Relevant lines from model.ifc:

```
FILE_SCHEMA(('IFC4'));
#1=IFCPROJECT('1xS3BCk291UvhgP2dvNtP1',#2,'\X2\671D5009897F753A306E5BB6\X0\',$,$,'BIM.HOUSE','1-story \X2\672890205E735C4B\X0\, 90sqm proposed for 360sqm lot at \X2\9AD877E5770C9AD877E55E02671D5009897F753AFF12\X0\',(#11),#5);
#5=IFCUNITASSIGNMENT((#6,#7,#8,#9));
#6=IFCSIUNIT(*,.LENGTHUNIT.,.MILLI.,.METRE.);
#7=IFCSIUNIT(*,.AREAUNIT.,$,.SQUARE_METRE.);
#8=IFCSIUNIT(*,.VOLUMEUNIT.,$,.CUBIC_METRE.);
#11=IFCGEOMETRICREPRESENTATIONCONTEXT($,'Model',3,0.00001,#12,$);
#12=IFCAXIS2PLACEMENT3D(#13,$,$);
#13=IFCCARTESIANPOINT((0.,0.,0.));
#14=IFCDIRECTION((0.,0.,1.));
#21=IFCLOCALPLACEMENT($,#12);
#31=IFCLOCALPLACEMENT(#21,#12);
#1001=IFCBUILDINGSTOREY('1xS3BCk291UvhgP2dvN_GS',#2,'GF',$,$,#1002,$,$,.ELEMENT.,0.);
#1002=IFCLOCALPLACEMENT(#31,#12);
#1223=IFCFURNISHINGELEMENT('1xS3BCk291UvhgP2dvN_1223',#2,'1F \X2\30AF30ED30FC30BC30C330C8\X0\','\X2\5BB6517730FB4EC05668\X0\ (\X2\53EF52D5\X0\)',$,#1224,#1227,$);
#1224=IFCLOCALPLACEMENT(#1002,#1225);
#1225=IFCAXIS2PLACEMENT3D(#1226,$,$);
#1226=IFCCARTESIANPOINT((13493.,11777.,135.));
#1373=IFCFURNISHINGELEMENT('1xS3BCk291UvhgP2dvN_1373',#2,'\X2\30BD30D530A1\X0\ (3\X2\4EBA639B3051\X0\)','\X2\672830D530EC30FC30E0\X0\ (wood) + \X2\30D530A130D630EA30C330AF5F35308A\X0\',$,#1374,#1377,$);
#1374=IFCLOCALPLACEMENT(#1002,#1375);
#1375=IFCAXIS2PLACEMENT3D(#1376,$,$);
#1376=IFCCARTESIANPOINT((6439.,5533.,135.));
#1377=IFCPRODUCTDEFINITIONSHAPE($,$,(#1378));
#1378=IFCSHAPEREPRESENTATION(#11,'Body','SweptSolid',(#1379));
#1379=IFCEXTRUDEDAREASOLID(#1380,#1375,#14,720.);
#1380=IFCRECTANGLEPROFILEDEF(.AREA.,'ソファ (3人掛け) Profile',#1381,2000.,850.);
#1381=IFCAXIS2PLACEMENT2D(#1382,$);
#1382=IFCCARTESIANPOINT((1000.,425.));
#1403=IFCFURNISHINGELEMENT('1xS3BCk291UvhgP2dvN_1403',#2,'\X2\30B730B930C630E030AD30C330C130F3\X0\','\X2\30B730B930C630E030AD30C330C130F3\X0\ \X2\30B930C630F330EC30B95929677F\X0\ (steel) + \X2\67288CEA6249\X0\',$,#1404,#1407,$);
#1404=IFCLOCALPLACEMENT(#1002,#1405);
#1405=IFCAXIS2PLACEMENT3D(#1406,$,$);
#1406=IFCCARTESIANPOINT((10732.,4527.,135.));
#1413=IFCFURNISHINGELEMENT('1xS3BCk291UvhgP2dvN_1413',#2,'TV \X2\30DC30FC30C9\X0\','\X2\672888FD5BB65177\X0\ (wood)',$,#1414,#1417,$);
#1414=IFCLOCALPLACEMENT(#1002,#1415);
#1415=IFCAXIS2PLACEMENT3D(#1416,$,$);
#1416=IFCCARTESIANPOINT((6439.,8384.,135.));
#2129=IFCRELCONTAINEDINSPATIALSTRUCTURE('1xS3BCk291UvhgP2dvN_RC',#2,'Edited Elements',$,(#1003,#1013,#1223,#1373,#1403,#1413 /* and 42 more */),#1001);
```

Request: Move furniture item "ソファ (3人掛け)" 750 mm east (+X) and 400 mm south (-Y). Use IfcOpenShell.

```python
import ifcopenshell
import ifcopenshell.api.geometry
import ifcopenshell.util.placement
import ifcopenshell.util.unit

model = ifcopenshell.open("model.ifc")
unit_scale = ifcopenshell.util.unit.calculate_unit_scale(model)

item = model.by_guid("1xS3BCk291UvhgP2dvN_1373")
matrix = ifcopenshell.util.placement.get_local_placement(item.ObjectPlacement)
matrix[0, 3] += 0.75 / unit_scale
matrix[1, 3] -= 0.4 / unit_scale
ifcopenshell.api.geometry.edit_object_placement(model, product=item, matrix=matrix, is_si=False)

print(ifcopenshell.util.placement.get_local_placement(item.ObjectPlacement).round(3) + 0.0)

model.write("model-out.ifc")
```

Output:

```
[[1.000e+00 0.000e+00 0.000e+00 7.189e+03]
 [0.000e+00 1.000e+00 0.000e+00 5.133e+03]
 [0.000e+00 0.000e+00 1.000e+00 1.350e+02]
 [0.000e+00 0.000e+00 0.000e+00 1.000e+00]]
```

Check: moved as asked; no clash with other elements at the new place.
